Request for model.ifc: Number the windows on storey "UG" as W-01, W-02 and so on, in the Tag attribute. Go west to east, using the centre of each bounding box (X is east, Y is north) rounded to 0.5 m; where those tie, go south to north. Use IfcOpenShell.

First a look at what the model holds.

```python
import ifcopenshell
import ifcopenshell.util.element
import ifcopenshell.util.placement

model = ifcopenshell.open("model.ifc")
print(model.schema)
storey = next(s for s in model.by_type("IfcBuildingStorey") if s.Name == "UG")
windows = [e for e in ifcopenshell.util.element.get_decomposition(storey) if e.is_a("IfcWindow")]
for e in sorted(windows, key=lambda e: e.id()):
    origin = ifcopenshell.util.placement.get_local_placement(e.ObjectPlacement)[:3, 3]
    print(e.id(), e.Tag, e.Name, origin.round(2) + 0.0, sep=" | ")
```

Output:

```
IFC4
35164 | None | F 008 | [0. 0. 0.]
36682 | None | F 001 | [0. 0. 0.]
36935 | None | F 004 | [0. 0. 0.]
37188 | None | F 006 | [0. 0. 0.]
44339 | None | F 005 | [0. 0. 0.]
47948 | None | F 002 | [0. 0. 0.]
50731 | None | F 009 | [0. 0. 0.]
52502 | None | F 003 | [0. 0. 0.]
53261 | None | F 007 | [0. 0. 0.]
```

```python
import ifcopenshell
import ifcopenshell.geom
import ifcopenshell.util.element
import ifcopenshell.util.shape

model = ifcopenshell.open("model.ifc")
settings = ifcopenshell.geom.settings()
settings.set("use-world-coords", True)


def centre(element):
    shape = ifcopenshell.geom.create_shape(settings, element)
    return ifcopenshell.util.shape.get_bbox_centroid(shape.geometry)


storey = next(s for s in model.by_type("IfcBuildingStorey") if s.Name == "UG")
windows = [e for e in ifcopenshell.util.element.get_decomposition(storey) if e.is_a("IfcWindow")]

# Insertion points can sit at a corner or the storey origin, so sort by the geometry (in metres).
centres = {e: centre(e) for e in windows}
windows.sort(key=lambda e: (round(centres[e][0] / 0.5), centres[e][1]))

for i, e in enumerate(windows, start=1):
    number = f"W-{i:02d}"
    e.Tag = number
    print(e.id(), number)

model.write("model-out.ifc")
```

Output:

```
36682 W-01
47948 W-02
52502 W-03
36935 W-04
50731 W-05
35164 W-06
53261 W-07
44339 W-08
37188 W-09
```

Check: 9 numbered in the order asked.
